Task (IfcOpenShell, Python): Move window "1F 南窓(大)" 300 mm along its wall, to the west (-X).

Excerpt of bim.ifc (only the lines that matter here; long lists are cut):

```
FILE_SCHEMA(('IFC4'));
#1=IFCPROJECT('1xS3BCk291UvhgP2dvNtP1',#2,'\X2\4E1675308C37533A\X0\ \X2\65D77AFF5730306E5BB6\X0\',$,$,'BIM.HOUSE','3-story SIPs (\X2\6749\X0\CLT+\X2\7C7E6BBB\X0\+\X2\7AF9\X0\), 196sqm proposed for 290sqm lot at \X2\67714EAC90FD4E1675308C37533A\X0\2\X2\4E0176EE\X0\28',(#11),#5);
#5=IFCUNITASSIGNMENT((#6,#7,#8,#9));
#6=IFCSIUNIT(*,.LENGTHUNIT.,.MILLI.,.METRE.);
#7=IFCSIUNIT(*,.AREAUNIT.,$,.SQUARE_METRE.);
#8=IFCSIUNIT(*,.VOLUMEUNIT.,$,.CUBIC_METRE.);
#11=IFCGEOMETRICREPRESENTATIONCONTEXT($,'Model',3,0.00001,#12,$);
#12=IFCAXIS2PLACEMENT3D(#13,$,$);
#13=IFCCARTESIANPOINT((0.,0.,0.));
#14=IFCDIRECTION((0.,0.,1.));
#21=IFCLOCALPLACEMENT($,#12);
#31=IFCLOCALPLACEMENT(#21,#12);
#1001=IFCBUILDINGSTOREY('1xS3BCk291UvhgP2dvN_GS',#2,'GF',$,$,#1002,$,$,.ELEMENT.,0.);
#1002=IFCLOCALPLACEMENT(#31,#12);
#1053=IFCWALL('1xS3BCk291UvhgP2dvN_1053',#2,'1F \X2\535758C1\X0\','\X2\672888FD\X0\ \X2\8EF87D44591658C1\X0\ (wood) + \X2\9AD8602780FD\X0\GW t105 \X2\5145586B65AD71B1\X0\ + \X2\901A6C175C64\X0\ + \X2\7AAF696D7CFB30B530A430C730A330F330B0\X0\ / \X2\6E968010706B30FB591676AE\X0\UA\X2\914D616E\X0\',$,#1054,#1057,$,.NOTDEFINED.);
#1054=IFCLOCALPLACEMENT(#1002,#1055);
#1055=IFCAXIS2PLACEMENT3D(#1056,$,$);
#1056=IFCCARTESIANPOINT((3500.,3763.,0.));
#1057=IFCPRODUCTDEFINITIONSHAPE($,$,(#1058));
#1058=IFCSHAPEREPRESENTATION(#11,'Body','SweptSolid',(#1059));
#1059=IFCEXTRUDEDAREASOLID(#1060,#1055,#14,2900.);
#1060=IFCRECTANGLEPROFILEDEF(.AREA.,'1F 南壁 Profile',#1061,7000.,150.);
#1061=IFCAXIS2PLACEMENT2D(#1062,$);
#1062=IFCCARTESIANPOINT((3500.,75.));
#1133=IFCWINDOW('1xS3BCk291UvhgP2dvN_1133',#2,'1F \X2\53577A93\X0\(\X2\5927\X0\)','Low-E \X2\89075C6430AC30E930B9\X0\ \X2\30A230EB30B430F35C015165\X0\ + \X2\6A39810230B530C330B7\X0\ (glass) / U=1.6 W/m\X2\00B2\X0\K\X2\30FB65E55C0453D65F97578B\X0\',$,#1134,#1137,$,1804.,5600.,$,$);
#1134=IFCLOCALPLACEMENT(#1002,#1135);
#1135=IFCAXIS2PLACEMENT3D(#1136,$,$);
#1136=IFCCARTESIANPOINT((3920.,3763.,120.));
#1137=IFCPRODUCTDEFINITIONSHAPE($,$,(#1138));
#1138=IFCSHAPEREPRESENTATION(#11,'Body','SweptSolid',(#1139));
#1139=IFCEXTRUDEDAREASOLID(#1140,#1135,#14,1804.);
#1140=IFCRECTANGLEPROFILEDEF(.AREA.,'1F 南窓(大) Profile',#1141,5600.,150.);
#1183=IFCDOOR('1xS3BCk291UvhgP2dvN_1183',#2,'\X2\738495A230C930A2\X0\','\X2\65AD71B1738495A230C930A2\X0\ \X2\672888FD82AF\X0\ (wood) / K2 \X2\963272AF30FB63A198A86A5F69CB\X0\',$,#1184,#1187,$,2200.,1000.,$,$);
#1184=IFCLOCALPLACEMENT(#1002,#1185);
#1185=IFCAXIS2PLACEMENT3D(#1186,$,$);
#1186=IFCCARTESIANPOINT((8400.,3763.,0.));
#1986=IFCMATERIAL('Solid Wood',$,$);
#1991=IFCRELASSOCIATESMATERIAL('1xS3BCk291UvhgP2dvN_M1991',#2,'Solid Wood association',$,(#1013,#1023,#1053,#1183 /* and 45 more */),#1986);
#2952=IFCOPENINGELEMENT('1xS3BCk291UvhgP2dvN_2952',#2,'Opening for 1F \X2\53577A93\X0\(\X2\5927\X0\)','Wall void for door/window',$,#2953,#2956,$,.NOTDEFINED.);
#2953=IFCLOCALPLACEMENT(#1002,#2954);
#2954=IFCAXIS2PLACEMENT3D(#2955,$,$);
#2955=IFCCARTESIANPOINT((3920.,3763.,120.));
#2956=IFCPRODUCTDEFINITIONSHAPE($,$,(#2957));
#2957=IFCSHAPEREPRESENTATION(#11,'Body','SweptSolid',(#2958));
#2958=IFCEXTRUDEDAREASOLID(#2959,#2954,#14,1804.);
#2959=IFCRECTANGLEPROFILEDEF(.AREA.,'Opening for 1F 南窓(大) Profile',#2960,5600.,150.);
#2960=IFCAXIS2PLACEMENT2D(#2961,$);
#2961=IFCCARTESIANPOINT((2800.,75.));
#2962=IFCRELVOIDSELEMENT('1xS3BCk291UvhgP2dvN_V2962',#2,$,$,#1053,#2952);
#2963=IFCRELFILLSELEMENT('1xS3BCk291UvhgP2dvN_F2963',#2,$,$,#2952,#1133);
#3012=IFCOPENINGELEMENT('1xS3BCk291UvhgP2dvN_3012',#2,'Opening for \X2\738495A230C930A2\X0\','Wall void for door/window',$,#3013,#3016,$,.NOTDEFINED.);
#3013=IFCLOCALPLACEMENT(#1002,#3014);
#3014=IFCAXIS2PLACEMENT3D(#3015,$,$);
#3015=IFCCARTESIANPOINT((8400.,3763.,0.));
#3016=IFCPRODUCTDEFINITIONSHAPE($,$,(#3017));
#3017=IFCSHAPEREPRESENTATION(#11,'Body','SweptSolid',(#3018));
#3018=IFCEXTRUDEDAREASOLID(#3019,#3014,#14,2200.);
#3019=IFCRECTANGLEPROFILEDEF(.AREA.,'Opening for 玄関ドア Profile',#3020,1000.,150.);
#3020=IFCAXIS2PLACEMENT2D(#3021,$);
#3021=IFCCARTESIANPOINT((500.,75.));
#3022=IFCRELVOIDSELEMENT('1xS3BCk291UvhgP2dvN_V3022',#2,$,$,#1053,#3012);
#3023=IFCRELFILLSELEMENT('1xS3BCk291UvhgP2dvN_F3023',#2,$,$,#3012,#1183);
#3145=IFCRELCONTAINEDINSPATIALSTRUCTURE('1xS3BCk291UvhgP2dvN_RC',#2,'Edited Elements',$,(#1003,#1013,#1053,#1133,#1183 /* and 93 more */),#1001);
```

```python
import ifcopenshell
import ifcopenshell.api.geometry
import ifcopenshell.util.placement
import ifcopenshell.util.unit

model = ifcopenshell.open("bim.ifc")
unit_scale = ifcopenshell.util.unit.calculate_unit_scale(model)

window = model.by_guid("1xS3BCk291UvhgP2dvN_1133")
opening = window.FillsVoids[0].RelatingOpeningElement
wall = opening.VoidsElements[0].RelatingBuildingElement

wall_matrix = ifcopenshell.util.placement.get_local_placement(wall.ObjectPlacement)
shift = wall_matrix[:3, 0] * -0.3 / unit_scale
before = ifcopenshell.util.placement.get_local_placement(window.ObjectPlacement)[:3, 3].copy()

# The window is not placed relative to its opening, so move both.
for product in (opening, window):
    matrix = ifcopenshell.util.placement.get_local_placement(product.ObjectPlacement)
    matrix[:3, 3] += shift
    ifcopenshell.api.geometry.edit_object_placement(model, product=product, matrix=matrix, is_si=False)

after = ifcopenshell.util.placement.get_local_placement(window.ObjectPlacement)[:3, 3]
print("window moved by", (after - before).round(3) + 0.0)

model.write("bim_edited.ifc")
```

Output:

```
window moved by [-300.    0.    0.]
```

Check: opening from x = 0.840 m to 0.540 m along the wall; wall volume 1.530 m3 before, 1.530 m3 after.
